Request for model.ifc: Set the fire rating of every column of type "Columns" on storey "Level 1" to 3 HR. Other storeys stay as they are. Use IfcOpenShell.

First a look at what the model holds.

```python
import ifcopenshell
import ifcopenshell.util.element

model = ifcopenshell.open("model.ifc")
print(model.schema)
storey = next(s for s in model.by_type("IfcBuildingStorey") if s.Name == "Level 1")
columns = [e for e in ifcopenshell.util.element.get_decomposition(storey) if e.is_a("IfcColumn")]
seen = {}
for e in columns:
    element_type = ifcopenshell.util.element.get_type(e)
    key = (element_type.Name if element_type != e and element_type else None, ifcopenshell.util.element.get_pset(e, "Pset_ColumnCommon", "FireRating"))
    seen[key] = seen.get(key, 0) + 1
for (name, value), count in sorted(seen.items(), key=str):
    print(count, "x", name, "|", value)
```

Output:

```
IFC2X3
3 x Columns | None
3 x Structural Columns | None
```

```python
import ifcopenshell
import ifcopenshell.api.pset
import ifcopenshell.util.element

model = ifcopenshell.open("model.ifc")

storey = next(s for s in model.by_type("IfcBuildingStorey") if s.Name == "Level 1")
columns = [e for e in ifcopenshell.util.element.get_decomposition(storey) if e.is_a("IfcColumn")]

count = 0
for e in columns:
    element_type = ifcopenshell.util.element.get_type(e)
    if element_type in (None, e) or element_type.Name != "Columns":
        continue
    # add_pset returns the element's existing set when there is one.
    pset = ifcopenshell.api.pset.add_pset(model, product=e, name="Pset_ColumnCommon")
    ifcopenshell.api.pset.edit_pset(model, pset=pset, properties={"FireRating": "3 HR"})
    count += 1

print(count, "columns updated")

model.write("model_rev.ifc")
```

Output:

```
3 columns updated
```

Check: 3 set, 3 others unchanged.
